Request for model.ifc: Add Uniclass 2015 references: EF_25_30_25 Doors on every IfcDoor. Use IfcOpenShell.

First a look at what the model holds.

```python
import ifcopenshell

model = ifcopenshell.open("model.ifc")
print(model.schema)
print("classifications:", [c.Name for c in model.by_type("IfcClassification")])
for ifc_class in ("IfcDoor", "IfcRoof", "IfcStair", "IfcWall", "IfcWindow"):
    print(ifc_class, len(model.by_type(ifc_class)))
```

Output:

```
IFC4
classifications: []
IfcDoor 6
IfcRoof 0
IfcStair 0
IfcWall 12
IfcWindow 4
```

```python
import ifcopenshell
import ifcopenshell.api.classification

model = ifcopenshell.open("model.ifc")

system = ifcopenshell.api.classification.add_classification(model, classification="Uniclass 2015")

codes = {
    "IfcDoor": ("EF_25_30_25", "Doors"),
}
for ifc_class, (code, name) in codes.items():
    products = model.by_type(ifc_class)
    ifcopenshell.api.classification.add_reference(
        model, products=products, classification=system, identification=code, name=name
    )
    print(code, len(products))

model.write("model-out.ifc")
```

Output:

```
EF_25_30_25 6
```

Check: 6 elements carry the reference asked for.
